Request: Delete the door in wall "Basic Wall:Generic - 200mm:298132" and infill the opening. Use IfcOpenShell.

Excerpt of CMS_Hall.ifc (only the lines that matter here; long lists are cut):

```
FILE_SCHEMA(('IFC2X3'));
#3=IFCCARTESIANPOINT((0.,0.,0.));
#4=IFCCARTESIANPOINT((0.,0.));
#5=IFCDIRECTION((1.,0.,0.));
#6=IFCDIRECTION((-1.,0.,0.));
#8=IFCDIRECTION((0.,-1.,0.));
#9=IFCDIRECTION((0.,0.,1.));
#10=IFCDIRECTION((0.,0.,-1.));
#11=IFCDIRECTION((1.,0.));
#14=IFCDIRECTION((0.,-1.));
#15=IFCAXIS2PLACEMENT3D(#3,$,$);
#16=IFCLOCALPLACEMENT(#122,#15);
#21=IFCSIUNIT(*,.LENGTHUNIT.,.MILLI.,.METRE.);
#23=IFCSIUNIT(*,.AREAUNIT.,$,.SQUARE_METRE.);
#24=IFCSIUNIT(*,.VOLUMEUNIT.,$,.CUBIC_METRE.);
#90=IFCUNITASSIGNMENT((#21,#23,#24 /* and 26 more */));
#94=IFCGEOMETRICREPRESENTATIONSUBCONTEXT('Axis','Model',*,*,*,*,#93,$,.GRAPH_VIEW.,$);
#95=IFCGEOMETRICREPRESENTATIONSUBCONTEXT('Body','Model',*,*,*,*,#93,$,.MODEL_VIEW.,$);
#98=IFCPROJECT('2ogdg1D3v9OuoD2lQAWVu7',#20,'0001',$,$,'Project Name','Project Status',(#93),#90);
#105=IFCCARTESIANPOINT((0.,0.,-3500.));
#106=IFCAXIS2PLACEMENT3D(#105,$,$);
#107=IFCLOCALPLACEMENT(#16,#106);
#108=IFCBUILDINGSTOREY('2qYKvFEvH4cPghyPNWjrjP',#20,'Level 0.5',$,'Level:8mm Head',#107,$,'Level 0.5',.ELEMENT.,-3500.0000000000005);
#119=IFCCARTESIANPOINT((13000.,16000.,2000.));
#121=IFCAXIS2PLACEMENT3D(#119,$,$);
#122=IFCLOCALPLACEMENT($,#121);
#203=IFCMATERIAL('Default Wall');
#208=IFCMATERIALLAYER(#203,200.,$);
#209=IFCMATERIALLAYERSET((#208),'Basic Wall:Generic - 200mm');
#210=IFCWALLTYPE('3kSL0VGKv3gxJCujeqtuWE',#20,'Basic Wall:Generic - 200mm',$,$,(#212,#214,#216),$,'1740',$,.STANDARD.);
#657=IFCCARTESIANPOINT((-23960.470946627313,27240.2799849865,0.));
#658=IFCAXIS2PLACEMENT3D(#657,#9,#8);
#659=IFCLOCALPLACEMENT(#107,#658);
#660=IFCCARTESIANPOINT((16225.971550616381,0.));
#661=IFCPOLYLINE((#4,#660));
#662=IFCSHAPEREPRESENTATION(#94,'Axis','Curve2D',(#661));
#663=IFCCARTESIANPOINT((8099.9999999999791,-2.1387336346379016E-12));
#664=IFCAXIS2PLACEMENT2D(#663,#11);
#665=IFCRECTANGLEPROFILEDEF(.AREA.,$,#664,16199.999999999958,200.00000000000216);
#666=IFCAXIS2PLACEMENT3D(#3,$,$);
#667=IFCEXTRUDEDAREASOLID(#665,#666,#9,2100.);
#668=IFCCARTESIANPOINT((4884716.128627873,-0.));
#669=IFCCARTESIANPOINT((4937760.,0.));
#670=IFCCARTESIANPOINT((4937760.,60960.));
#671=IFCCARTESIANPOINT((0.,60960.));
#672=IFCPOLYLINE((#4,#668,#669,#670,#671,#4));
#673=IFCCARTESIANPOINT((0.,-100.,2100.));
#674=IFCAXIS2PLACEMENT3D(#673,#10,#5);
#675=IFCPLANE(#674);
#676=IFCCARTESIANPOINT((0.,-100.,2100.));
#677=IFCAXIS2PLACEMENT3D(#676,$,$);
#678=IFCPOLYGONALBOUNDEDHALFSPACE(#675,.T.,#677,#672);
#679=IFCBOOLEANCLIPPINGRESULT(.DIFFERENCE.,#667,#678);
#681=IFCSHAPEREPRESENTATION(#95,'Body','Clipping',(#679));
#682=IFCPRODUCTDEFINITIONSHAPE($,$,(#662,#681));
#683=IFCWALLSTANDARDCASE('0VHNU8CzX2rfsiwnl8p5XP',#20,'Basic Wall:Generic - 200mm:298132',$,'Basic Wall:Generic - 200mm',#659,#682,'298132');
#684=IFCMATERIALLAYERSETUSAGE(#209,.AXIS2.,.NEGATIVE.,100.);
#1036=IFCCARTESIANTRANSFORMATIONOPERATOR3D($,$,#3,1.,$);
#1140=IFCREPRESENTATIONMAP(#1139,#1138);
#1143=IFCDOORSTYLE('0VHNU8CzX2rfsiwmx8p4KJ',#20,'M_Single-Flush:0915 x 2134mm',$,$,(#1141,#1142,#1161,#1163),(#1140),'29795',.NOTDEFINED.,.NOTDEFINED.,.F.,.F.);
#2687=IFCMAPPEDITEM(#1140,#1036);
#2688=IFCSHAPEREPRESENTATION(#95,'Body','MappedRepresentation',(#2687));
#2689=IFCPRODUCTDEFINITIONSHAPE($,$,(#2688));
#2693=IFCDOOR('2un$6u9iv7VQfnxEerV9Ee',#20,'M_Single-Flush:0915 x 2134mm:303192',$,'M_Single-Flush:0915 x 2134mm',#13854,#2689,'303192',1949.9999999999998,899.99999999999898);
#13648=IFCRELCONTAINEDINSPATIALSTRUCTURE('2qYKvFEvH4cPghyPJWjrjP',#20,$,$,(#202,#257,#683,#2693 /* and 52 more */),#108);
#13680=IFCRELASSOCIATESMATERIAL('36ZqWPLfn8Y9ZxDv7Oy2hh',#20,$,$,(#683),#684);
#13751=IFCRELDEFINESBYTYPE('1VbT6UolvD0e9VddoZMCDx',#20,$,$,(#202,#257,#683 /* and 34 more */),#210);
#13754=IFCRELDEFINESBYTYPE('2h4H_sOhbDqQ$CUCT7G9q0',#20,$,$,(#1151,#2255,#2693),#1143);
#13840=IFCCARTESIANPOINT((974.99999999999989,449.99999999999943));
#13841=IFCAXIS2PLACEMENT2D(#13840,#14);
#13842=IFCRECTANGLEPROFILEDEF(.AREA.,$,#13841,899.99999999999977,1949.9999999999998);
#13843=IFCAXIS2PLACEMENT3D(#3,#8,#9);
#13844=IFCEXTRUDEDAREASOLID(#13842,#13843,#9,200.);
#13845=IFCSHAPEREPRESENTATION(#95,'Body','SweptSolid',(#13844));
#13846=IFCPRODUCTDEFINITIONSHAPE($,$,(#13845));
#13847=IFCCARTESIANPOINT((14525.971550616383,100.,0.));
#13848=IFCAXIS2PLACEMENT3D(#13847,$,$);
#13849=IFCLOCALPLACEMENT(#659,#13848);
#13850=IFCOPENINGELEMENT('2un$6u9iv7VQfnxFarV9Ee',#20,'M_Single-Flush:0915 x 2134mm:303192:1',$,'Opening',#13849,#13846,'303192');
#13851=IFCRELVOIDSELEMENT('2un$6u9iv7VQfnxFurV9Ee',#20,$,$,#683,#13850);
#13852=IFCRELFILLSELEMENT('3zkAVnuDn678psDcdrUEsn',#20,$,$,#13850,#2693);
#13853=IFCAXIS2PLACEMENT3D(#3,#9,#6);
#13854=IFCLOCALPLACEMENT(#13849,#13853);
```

```python
import ifcopenshell
import ifcopenshell.api.feature
import ifcopenshell.api.root
import ifcopenshell.geom
import ifcopenshell.util.shape

model = ifcopenshell.open("CMS_Hall.ifc")
settings = ifcopenshell.geom.settings()


def volume(element):
    """Net volume in cubic metres, openings subtracted."""
    shape = ifcopenshell.geom.create_shape(settings, element)
    return ifcopenshell.util.shape.get_volume(shape.geometry)


door = model.by_id(2693)
opening = door.FillsVoids[0].RelatingOpeningElement
wall = opening.VoidsElements[0].RelatingBuildingElement
before = volume(wall)

ifcopenshell.api.root.remove_product(model, product=door)
ifcopenshell.api.feature.remove_feature(model, feature=opening)

after = volume(wall)

print(f"wall volume {before:.3f} -> {after:.3f} m3")

model.write("CMS_Hall_updated.ifc")
```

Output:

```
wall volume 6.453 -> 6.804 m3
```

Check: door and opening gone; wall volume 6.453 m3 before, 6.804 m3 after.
